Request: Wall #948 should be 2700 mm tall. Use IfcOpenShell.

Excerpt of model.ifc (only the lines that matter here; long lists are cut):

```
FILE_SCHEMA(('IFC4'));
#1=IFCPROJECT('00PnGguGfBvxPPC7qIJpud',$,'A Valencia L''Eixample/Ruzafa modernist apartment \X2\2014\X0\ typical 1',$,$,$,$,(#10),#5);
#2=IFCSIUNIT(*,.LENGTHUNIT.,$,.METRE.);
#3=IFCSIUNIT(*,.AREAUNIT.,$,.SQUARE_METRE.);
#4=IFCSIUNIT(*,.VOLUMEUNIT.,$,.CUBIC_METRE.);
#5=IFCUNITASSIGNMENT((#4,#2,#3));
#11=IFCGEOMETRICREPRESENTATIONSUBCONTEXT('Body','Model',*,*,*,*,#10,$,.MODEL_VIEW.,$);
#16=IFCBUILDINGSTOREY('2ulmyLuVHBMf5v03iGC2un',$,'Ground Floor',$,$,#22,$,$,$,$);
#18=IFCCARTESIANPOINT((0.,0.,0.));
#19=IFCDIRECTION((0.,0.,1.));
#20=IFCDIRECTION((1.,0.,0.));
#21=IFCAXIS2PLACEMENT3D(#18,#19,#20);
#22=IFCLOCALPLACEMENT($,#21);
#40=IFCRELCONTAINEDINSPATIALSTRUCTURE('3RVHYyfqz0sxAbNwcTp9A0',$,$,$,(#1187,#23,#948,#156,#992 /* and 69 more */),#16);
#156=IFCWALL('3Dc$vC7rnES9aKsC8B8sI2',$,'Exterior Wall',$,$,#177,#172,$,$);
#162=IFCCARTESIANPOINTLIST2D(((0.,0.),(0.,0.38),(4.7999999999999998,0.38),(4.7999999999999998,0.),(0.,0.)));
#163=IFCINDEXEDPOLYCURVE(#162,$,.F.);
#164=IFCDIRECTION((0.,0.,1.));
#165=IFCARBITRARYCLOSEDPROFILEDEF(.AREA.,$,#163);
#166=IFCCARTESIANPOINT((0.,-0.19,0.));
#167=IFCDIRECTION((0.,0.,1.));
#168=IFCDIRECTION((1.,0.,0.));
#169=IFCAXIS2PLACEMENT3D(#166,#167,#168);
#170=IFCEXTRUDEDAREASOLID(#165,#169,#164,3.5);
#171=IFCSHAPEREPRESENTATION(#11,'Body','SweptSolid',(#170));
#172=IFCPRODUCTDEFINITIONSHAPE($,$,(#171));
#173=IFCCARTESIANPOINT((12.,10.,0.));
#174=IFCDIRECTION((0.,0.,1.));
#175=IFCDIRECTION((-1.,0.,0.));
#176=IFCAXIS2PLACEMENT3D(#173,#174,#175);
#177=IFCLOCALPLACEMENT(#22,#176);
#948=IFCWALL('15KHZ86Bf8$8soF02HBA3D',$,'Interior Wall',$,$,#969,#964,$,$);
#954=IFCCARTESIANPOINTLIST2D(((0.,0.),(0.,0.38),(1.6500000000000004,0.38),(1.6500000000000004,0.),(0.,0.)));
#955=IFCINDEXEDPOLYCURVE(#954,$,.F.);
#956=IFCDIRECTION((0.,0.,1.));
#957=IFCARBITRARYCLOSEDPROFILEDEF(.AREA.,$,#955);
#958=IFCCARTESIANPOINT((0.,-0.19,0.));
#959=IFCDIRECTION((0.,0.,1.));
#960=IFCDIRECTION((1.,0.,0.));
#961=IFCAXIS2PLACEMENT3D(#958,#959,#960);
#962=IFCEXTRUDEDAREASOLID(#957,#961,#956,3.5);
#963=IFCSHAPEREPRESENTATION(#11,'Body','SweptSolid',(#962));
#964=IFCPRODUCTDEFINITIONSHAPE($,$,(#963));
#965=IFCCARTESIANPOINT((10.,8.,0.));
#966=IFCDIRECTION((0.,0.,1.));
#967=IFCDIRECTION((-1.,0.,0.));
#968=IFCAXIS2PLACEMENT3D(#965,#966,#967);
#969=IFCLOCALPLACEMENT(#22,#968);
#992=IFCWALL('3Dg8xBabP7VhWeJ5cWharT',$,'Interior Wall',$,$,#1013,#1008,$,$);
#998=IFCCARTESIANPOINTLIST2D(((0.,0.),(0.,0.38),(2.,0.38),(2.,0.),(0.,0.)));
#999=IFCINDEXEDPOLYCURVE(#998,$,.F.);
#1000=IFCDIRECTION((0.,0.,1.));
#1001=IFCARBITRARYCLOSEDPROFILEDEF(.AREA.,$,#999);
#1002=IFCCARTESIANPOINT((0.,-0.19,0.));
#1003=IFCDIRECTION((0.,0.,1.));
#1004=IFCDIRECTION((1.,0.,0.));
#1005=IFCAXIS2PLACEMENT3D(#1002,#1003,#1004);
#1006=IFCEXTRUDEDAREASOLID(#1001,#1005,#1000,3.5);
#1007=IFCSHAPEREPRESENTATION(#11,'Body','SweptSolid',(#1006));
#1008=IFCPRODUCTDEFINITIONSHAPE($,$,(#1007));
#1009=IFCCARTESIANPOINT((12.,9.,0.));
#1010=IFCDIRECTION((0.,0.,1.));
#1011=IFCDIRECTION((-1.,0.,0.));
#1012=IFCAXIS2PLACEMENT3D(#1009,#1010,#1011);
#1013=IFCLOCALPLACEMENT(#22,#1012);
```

```python
import ifcopenshell
import ifcopenshell.geom
import ifcopenshell.util.representation
import ifcopenshell.util.shape
import ifcopenshell.util.unit

model = ifcopenshell.open("model.ifc")
unit_scale = ifcopenshell.util.unit.calculate_unit_scale(model)
settings = ifcopenshell.geom.settings()


def volume(element):
    """Net volume in cubic metres, openings subtracted."""
    shape = ifcopenshell.geom.create_shape(settings, element)
    return ifcopenshell.util.shape.get_volume(shape.geometry)


wall = model.by_id(948)
before = volume(wall)

body = ifcopenshell.util.representation.get_representation(wall, "Model", "Body")
solid = body.Items[0]
old_height = solid.Depth
solid.Depth = 2.7 / unit_scale
after = volume(wall)

print(f"height {old_height:g} -> {solid.Depth:g}, volume {before:.3f} -> {after:.3f} m3")

model.write("model-out.ifc")
```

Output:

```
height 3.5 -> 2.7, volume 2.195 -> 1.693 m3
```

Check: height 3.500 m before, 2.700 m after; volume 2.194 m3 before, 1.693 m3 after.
